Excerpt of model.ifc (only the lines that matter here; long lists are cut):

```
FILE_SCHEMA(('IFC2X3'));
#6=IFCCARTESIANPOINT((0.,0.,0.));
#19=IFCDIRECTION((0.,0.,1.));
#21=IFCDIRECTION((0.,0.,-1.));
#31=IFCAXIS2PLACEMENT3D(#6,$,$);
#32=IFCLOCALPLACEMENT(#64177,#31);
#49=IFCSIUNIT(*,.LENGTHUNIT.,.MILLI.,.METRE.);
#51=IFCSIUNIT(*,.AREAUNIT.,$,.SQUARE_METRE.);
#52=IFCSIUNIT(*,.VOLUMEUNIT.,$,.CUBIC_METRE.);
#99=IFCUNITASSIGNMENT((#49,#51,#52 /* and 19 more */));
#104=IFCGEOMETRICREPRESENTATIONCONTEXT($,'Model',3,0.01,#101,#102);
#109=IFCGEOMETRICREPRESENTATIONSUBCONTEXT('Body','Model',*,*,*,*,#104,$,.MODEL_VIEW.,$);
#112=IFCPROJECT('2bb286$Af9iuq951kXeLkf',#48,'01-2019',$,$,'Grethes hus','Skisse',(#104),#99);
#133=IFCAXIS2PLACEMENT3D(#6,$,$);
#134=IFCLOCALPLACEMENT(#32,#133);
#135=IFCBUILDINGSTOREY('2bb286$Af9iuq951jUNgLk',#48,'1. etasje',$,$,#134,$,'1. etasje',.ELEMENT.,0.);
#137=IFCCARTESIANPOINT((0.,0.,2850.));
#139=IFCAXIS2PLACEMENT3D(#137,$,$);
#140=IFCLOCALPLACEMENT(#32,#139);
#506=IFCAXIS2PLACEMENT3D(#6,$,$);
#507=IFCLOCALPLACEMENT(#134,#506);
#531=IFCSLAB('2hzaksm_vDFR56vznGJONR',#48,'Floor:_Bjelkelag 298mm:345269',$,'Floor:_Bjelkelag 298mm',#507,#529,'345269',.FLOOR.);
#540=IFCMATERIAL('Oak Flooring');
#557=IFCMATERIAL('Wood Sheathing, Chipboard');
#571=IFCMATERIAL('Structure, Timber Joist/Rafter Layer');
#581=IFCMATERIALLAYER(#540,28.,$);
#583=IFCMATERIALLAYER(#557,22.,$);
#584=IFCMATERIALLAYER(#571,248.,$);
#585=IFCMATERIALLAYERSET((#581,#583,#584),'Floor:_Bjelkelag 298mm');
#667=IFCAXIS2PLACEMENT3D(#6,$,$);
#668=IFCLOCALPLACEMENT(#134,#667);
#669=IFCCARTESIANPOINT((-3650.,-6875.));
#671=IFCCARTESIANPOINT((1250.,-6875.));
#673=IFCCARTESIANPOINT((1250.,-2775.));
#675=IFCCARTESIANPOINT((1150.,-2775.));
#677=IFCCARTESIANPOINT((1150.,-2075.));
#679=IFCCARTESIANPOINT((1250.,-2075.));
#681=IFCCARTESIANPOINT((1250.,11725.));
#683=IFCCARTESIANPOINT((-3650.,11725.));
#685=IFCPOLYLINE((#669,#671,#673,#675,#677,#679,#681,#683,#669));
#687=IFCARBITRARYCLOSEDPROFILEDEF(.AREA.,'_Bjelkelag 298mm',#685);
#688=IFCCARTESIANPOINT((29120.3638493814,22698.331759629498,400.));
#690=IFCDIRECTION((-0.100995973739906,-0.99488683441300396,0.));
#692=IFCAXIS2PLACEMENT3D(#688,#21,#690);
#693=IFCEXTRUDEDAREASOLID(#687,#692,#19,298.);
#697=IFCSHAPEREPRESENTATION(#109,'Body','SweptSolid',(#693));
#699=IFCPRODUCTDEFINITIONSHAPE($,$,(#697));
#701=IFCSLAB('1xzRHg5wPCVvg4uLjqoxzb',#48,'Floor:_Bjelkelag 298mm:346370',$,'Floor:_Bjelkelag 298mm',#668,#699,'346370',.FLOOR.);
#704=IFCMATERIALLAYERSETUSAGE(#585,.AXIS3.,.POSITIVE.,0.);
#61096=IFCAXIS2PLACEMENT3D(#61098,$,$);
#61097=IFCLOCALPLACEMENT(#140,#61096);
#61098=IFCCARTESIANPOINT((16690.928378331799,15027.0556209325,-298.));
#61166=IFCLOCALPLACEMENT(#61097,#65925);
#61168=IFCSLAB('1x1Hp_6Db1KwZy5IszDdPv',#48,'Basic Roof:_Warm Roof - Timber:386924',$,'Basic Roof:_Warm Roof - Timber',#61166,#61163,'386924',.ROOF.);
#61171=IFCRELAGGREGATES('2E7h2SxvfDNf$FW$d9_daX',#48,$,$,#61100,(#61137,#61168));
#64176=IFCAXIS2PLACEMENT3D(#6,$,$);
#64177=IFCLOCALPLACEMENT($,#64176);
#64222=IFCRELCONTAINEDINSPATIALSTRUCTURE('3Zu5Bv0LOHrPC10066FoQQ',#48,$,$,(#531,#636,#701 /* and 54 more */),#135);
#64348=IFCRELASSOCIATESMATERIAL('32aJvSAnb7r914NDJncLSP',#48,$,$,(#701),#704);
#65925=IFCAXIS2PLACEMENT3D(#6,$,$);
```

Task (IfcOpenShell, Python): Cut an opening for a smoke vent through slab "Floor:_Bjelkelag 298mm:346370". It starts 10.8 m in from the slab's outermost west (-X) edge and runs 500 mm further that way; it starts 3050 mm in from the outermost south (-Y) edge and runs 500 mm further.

```python
import numpy as np
import ifcopenshell
import ifcopenshell.api.feature
import ifcopenshell.api.geometry
import ifcopenshell.api.root
import ifcopenshell.geom
import ifcopenshell.util.placement
import ifcopenshell.util.representation
import ifcopenshell.util.shape
import ifcopenshell.util.unit

model = ifcopenshell.open("model.ifc")
unit_scale = ifcopenshell.util.unit.calculate_unit_scale(model)
settings = ifcopenshell.geom.settings()


def volume(element):
    """Net volume in cubic metres, openings subtracted."""
    shape = ifcopenshell.geom.create_shape(settings, element)
    return ifcopenshell.util.shape.get_volume(shape.geometry)


slab = model.by_guid("1xzRHg5wPCVvg4uLjqoxzb")
before = volume(slab)

# Extent in the slab's own axes, in metres. The edges named are its -X and -Y sides.
slab_shape = ifcopenshell.geom.create_shape(settings, slab)
vertices = ifcopenshell.util.shape.get_vertices(slab_shape.geometry)
x_min, y_min, bottom = vertices.min(axis=0)
top = vertices[:, 2].max()

opening = ifcopenshell.api.root.create_entity(model, ifc_class="IfcOpeningElement", name="Smoke vent opening")
context = ifcopenshell.util.representation.get_context(model, "Model", "Body", "MODEL_VIEW")
width, depth = 0.5, 0.5
outline = [(0.0, 0.0), (width, 0.0), (width, depth), (0.0, depth), (0.0, 0.0)]
# Overshoot both faces by 50 mm so the cut is clean.
shape = ifcopenshell.api.geometry.add_slab_representation(
    model, context=context, depth=top - bottom + 0.1, polyline=outline
)
ifcopenshell.api.geometry.assign_representation(model, product=opening, representation=shape)

matrix = ifcopenshell.util.placement.get_local_placement(slab.ObjectPlacement)
matrix[:, 3] = matrix @ np.append(np.array([x_min + 10.8, y_min + 3.05, bottom - 0.05]) / unit_scale, 1.0)
ifcopenshell.api.geometry.edit_object_placement(model, product=opening, matrix=matrix, is_si=False)
ifcopenshell.api.feature.add_feature(model, feature=opening, element=slab)

after = volume(slab)

print(f"slab volume {before:.3f} -> {after:.3f} m3")

model.write("model-out.ifc")
```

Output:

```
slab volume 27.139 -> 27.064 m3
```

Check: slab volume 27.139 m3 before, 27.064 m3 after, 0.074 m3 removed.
